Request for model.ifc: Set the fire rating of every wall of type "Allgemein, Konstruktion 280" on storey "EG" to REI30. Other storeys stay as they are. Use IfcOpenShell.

First a look at what the model holds.

```python
import ifcopenshell
import ifcopenshell.util.element

model = ifcopenshell.open("model.ifc")
print(model.schema)
storey = next(s for s in model.by_type("IfcBuildingStorey") if s.Name == "EG")
walls = [e for e in ifcopenshell.util.element.get_decomposition(storey) if e.is_a("IfcWall")]
seen = {}
for e in walls:
    element_type = ifcopenshell.util.element.get_type(e)
    key = (element_type.Name if element_type != e and element_type else None, ifcopenshell.util.element.get_pset(e, "Pset_WallCommon", "FireRating"))
    seen[key] = seen.get(key, 0) + 1
for (name, value), count in sorted(seen.items(), key=str):
    print(count, "x", name, "|", value)
```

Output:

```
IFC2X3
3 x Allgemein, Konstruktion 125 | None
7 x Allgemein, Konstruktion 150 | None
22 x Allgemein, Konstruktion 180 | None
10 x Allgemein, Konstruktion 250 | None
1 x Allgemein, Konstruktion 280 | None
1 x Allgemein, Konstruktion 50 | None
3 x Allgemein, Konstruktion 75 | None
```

```python
import ifcopenshell
import ifcopenshell.api.pset
import ifcopenshell.util.element

model = ifcopenshell.open("model.ifc")

storey = next(s for s in model.by_type("IfcBuildingStorey") if s.Name == "EG")
walls = [e for e in ifcopenshell.util.element.get_decomposition(storey) if e.is_a("IfcWall")]

count = 0
for e in walls:
    element_type = ifcopenshell.util.element.get_type(e)
    if element_type in (None, e) or element_type.Name != "Allgemein, Konstruktion 280":
        continue
    # add_pset returns the element's existing set when there is one.
    pset = ifcopenshell.api.pset.add_pset(model, product=e, name="Pset_WallCommon")
    ifcopenshell.api.pset.edit_pset(model, pset=pset, properties={"FireRating": "REI30"})
    count += 1

print(count, "walls updated")

model.write("model_rev.ifc")
```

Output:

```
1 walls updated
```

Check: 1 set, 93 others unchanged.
